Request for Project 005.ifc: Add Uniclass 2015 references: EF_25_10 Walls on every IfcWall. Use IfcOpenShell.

First a look at what the model holds.

```python
import ifcopenshell

model = ifcopenshell.open("Project 005.ifc")
print(model.schema)
print("classifications:", [c.Name for c in model.by_type("IfcClassification")])
for ifc_class in ("IfcDoor", "IfcRoof", "IfcStair", "IfcWall", "IfcWindow"):
    print(ifc_class, len(model.by_type(ifc_class)))
```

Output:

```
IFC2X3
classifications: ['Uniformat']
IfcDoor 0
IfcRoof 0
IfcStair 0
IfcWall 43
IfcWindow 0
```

```python
import ifcopenshell
import ifcopenshell.api.classification

model = ifcopenshell.open("Project 005.ifc")

# IFC2X3 requires Source and Edition and has no link from the project to the system.
system = model.create_entity("IfcClassification", Source="NBS", Edition="2015", Name="Uniclass 2015")

codes = {
    "IfcWall": ("EF_25_10", "Walls"),
}
for ifc_class, (code, name) in codes.items():
    products = model.by_type(ifc_class)
    ifcopenshell.api.classification.add_reference(
        model, products=products, classification=system, identification=code, name=name
    )
    print(code, len(products))

model.write("Project 005_edited.ifc")
```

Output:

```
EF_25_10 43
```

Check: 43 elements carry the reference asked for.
